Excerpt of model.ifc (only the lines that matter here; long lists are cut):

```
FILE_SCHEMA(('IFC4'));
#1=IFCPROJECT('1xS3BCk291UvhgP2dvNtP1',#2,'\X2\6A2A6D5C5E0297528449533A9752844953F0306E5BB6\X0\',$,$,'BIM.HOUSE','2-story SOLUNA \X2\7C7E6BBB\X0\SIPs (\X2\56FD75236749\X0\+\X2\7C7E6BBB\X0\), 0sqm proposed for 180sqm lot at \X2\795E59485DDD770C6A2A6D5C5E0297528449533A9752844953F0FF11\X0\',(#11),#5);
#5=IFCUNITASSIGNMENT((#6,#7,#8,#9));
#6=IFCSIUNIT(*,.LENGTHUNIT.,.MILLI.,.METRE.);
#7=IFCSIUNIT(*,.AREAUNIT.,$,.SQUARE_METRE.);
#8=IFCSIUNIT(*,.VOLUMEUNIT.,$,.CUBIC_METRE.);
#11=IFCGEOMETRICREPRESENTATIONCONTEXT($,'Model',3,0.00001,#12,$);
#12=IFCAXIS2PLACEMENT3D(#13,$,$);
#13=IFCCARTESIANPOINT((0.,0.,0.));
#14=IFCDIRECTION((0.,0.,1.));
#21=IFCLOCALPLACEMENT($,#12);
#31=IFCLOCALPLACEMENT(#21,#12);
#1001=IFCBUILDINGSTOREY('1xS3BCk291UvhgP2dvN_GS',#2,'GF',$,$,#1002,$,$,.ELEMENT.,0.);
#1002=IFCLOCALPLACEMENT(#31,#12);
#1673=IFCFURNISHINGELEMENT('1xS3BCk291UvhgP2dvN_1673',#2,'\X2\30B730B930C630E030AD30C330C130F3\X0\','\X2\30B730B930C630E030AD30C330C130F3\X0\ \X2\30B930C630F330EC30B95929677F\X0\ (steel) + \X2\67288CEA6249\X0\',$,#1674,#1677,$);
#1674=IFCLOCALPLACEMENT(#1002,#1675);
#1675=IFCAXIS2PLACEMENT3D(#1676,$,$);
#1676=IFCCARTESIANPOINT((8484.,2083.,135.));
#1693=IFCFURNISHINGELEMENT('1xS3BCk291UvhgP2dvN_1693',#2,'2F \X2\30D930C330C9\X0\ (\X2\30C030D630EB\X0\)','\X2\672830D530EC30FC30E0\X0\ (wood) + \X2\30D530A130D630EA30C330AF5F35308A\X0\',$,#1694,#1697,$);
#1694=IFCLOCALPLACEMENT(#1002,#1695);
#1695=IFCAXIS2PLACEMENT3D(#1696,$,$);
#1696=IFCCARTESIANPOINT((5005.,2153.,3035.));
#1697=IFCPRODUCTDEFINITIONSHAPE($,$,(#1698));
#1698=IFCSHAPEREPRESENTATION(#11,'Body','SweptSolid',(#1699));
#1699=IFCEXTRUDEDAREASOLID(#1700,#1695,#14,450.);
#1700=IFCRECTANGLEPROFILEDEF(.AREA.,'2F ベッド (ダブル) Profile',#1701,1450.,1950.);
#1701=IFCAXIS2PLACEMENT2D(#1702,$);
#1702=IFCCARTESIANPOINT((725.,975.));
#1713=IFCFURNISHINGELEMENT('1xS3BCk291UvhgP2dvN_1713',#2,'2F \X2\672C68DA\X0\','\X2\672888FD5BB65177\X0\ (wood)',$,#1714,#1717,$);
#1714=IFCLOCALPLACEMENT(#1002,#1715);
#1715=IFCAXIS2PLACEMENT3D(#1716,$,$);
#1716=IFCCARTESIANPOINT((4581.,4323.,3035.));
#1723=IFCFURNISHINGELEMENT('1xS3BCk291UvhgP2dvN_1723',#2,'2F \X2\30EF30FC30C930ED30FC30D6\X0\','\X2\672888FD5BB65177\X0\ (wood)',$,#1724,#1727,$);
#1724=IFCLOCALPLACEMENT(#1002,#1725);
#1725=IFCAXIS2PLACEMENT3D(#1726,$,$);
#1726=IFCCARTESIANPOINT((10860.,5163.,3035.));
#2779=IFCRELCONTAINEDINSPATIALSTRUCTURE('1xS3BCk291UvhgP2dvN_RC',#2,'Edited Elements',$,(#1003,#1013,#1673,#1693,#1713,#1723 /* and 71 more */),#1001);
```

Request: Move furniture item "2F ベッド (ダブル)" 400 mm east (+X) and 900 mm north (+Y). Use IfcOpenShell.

```python
import ifcopenshell
import ifcopenshell.api.geometry
import ifcopenshell.util.placement

model = ifcopenshell.open("model.ifc")

item = model.by_id(1693)
matrix = ifcopenshell.util.placement.get_local_placement(item.ObjectPlacement)
matrix[0, 3] += 400.0
matrix[1, 3] += 900.0
ifcopenshell.api.geometry.edit_object_placement(model, product=item, matrix=matrix, is_si=False)

print(ifcopenshell.util.placement.get_local_placement(item.ObjectPlacement).round(3) + 0.0)

model.write("model-out.ifc")
```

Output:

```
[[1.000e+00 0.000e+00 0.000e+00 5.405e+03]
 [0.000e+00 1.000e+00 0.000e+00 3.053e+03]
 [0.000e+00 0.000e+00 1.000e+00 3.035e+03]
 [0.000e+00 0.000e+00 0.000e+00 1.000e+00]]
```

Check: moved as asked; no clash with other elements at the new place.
